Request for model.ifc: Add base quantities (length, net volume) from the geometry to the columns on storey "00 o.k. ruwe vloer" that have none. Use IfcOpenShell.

First a look at what the model holds.

```python
import ifcopenshell
import ifcopenshell.util.element
import ifcopenshell.util.unit

model = ifcopenshell.open("model.ifc")
print(model.schema)
for unit_type in ("LENGTHUNIT", "AREAUNIT", "VOLUMEUNIT"):
    print(unit_type, ifcopenshell.util.unit.calculate_unit_scale(model, unit_type))
storey = next(s for s in model.by_type("IfcBuildingStorey") if s.Name == "00 o.k. ruwe vloer")
columns = [e for e in ifcopenshell.util.element.get_decomposition(storey) if e.is_a("IfcColumn")]
for e in sorted(columns, key=lambda e: e.id()):
    print(e.id(), e.is_a(), e.Name, list(ifcopenshell.util.element.get_psets(e, qtos_only=True)), sep=" | ")
```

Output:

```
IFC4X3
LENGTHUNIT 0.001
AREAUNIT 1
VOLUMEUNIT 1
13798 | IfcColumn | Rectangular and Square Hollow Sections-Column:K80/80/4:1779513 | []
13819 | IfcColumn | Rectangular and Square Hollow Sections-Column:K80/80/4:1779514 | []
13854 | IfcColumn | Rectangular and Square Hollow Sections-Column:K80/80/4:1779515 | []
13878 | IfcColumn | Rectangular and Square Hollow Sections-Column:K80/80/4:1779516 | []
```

```python
import ifcopenshell
import ifcopenshell.api.pset
import ifcopenshell.geom
import ifcopenshell.util.element
import ifcopenshell.util.shape
import ifcopenshell.util.unit

model = ifcopenshell.open("model.ifc")
unit_scale = ifcopenshell.util.unit.calculate_unit_scale(model)
volume_scale = ifcopenshell.util.unit.calculate_unit_scale(model, "VOLUMEUNIT")
settings = ifcopenshell.geom.settings()

storey = next(s for s in model.by_type("IfcBuildingStorey") if s.Name == "00 o.k. ruwe vloer")
columns = [e for e in ifcopenshell.util.element.get_decomposition(storey) if e.is_a("IfcColumn")]

for e in sorted(columns, key=lambda e: e.id()):
    if ifcopenshell.util.element.get_psets(e, qtos_only=True, should_inherit=False):
        continue
    # Geometry comes back in metres, in the element's own axes.
    shape = ifcopenshell.geom.create_shape(settings, e)
    values = {
        "Length": ifcopenshell.util.shape.get_z(shape.geometry) / unit_scale,
        "NetVolume": ifcopenshell.util.shape.get_volume(shape.geometry) / volume_scale,
    }
    qto = ifcopenshell.api.pset.add_qto(model, product=e, name="Qto_ColumnBaseQuantities")
    ifcopenshell.api.pset.edit_qto(model, qto=qto, properties=values)
    print(e.id(), {k: round(v, 3) for k, v in values.items()})

model.write("model-out.ifc")
```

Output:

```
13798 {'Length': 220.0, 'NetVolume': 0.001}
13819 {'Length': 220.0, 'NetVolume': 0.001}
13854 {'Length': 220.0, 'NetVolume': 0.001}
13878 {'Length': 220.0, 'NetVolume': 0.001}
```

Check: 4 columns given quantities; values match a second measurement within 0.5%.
